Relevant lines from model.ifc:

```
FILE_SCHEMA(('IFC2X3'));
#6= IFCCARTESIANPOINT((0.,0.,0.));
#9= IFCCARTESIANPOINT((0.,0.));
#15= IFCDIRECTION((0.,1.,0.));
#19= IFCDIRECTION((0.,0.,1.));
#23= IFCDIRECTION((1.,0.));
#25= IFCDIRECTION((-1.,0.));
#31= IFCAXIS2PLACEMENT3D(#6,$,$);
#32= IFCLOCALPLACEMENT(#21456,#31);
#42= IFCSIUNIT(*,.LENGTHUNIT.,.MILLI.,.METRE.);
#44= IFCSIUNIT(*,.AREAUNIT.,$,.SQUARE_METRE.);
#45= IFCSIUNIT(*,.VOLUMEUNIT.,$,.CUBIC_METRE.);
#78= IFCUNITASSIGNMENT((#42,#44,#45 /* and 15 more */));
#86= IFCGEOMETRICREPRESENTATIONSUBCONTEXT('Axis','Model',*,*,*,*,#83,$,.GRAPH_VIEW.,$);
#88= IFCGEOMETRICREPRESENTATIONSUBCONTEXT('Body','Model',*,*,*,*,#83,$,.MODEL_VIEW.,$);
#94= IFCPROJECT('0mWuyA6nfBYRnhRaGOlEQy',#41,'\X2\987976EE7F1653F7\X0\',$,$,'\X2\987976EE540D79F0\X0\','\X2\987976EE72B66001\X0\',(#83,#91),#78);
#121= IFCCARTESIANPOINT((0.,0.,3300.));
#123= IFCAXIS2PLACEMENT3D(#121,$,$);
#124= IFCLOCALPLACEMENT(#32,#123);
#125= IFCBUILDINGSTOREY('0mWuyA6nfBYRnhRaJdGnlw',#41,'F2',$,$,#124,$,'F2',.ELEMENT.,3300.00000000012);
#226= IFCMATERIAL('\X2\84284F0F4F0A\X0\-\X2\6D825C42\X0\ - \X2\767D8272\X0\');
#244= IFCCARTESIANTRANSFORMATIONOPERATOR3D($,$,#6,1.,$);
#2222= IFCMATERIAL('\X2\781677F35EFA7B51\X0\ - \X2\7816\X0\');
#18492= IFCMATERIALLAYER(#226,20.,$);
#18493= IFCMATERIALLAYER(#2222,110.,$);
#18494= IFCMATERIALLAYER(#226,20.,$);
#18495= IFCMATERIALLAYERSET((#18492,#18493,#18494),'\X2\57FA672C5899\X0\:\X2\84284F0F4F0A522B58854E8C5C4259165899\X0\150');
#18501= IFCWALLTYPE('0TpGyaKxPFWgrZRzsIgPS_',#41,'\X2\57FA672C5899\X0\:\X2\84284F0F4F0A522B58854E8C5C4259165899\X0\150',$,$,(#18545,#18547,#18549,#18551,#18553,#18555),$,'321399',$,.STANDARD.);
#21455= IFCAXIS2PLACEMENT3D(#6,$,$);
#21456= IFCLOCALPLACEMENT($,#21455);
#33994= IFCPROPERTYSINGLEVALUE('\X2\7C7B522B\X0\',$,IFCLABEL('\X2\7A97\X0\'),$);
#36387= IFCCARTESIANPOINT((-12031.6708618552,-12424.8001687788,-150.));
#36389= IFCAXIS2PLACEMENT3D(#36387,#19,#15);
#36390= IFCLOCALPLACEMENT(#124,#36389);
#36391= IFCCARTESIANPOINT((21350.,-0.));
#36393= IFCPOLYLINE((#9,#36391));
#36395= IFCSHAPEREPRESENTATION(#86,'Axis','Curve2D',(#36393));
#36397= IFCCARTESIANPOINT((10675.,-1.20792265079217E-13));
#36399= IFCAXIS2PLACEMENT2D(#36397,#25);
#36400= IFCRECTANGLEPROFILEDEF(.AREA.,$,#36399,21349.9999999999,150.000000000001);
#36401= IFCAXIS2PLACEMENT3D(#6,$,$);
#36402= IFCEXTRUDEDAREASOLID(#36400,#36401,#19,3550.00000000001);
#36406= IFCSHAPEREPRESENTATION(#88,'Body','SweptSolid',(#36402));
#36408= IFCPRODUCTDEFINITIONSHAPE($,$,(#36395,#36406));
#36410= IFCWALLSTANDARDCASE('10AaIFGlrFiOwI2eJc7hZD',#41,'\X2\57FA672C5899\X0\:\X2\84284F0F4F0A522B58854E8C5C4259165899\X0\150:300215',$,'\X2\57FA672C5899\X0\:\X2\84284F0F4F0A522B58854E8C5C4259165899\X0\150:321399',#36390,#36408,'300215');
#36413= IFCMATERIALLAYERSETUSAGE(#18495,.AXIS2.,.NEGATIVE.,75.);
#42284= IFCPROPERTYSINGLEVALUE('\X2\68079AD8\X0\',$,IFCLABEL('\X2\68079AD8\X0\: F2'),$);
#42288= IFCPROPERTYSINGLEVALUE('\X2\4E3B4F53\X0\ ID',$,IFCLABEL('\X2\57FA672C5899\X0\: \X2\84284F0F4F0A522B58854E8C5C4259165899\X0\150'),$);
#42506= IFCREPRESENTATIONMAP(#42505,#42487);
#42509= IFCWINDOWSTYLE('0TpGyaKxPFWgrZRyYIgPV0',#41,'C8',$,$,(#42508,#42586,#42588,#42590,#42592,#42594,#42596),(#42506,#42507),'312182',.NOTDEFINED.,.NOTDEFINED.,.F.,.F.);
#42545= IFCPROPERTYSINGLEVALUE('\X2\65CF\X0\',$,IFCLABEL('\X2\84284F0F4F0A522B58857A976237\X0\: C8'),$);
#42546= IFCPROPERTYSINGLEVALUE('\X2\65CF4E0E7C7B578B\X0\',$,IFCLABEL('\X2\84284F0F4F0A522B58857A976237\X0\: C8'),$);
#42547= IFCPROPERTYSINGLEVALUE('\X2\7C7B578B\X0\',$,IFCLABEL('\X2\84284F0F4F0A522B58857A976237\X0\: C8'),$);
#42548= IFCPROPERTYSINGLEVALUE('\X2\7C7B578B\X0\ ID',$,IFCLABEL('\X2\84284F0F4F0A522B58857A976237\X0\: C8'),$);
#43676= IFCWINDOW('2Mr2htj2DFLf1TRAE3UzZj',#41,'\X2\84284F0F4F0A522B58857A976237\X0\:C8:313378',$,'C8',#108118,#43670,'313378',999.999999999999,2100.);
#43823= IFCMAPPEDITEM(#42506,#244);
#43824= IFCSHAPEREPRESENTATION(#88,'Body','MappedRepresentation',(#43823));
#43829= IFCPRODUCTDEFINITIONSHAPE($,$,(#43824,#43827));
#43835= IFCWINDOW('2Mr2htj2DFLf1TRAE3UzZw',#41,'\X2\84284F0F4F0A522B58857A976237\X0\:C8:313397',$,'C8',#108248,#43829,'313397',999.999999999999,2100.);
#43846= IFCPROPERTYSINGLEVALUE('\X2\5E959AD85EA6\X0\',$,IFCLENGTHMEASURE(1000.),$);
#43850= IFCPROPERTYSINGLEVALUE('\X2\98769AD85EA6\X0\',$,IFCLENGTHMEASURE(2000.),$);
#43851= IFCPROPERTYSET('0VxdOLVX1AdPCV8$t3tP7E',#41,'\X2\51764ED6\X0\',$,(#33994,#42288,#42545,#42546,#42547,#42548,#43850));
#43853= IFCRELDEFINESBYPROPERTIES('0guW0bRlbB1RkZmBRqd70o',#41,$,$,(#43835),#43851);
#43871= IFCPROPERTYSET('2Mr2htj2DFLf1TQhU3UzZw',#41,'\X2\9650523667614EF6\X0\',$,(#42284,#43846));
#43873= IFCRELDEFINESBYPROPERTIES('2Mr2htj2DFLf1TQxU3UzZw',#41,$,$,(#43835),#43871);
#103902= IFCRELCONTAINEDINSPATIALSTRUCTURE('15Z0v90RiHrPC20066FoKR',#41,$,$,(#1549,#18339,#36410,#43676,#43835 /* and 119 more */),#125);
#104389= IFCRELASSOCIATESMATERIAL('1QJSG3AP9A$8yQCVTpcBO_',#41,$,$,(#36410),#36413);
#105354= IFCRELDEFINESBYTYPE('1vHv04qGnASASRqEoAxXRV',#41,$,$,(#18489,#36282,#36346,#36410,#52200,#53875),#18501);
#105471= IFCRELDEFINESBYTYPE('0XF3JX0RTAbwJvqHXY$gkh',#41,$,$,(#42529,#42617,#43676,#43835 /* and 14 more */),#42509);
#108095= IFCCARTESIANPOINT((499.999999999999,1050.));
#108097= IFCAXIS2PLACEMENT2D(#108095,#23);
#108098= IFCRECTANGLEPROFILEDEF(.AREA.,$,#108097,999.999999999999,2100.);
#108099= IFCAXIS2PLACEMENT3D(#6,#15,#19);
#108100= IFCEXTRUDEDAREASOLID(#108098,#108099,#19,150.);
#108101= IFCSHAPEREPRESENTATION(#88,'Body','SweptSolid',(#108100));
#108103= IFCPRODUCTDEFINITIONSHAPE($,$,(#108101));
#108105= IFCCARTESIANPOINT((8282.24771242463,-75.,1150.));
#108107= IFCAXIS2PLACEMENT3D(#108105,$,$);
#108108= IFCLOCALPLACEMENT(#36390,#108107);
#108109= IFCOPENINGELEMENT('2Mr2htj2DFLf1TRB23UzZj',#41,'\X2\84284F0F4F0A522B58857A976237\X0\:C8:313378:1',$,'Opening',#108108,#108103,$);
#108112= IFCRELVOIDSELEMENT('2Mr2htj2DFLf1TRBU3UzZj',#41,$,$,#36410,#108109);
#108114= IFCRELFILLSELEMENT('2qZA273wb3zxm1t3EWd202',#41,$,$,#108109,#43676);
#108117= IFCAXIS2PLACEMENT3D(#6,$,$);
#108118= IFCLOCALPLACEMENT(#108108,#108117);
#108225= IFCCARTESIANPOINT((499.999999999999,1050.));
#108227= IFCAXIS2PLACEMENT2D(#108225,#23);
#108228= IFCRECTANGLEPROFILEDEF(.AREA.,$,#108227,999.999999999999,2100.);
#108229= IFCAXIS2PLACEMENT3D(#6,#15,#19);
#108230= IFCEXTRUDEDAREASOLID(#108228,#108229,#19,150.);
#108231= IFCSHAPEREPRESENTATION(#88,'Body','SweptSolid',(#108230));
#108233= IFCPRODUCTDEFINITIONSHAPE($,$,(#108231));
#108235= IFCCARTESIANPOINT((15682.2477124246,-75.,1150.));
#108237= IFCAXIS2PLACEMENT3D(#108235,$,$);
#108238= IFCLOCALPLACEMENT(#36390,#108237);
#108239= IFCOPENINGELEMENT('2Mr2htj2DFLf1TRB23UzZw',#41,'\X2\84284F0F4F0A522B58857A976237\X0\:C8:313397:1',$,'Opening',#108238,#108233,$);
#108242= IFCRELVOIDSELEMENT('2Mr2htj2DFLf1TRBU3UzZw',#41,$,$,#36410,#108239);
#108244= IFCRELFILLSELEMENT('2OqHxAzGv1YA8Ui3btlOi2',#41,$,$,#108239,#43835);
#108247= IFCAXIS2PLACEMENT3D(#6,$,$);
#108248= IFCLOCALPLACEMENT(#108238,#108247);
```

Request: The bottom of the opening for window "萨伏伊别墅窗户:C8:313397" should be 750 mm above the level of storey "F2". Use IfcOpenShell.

```python
import numpy as np
import ifcopenshell
import ifcopenshell.api.geometry
import ifcopenshell.api.pset
import ifcopenshell.geom
import ifcopenshell.util.element
import ifcopenshell.util.placement
import ifcopenshell.util.shape
import ifcopenshell.util.unit

model = ifcopenshell.open("model.ifc")
unit_scale = ifcopenshell.util.unit.calculate_unit_scale(model)

window = model.by_guid("2Mr2htj2DFLf1TRAE3UzZw")
opening = window.FillsVoids[0].RelatingOpeningElement
storey = ifcopenshell.util.element.get_container(window, ifc_class="IfcBuildingStorey")
level = ifcopenshell.util.placement.get_local_placement(storey.ObjectPlacement)[2, 3]

# The opening's origin need not be at the sill, so measure its lowest point.
shape = ifcopenshell.geom.create_shape(ifcopenshell.geom.settings(), opening)
bottom = ifcopenshell.util.shape.get_shape_bottom_elevation(shape, shape.geometry) / unit_scale
dz = level + 0.75 / unit_scale - bottom

shift = np.array([0.0, 0.0, dz])
# The window is placed relative to its opening, so it follows when the opening moves.
matrix = ifcopenshell.util.placement.get_local_placement(opening.ObjectPlacement)
matrix[:3, 3] += shift
ifcopenshell.api.geometry.edit_object_placement(
    model, product=opening, matrix=matrix, is_si=False, should_transform_children=True
)

# Keep the stored heights in step.
pset = model.by_id(ifcopenshell.util.element.get_pset(window, "其他", should_inherit=False)["id"])
ifcopenshell.api.pset.edit_pset(model, pset=pset, properties={
    "顶高度": model.create_entity("IfcLengthMeasure", ifcopenshell.util.element.get_pset(window, "其他", "顶高度") + dz),
})
pset = model.by_id(ifcopenshell.util.element.get_pset(window, "限制条件", should_inherit=False)["id"])
ifcopenshell.api.pset.edit_pset(model, pset=pset, properties={
    "底高度": model.create_entity("IfcLengthMeasure", ifcopenshell.util.element.get_pset(window, "限制条件", "底高度") + dz),
})

print(f"moved by {dz * unit_scale:+.3f} m")

model.write("model-out.ifc")
```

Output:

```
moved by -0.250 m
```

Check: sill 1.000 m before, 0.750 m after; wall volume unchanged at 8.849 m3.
